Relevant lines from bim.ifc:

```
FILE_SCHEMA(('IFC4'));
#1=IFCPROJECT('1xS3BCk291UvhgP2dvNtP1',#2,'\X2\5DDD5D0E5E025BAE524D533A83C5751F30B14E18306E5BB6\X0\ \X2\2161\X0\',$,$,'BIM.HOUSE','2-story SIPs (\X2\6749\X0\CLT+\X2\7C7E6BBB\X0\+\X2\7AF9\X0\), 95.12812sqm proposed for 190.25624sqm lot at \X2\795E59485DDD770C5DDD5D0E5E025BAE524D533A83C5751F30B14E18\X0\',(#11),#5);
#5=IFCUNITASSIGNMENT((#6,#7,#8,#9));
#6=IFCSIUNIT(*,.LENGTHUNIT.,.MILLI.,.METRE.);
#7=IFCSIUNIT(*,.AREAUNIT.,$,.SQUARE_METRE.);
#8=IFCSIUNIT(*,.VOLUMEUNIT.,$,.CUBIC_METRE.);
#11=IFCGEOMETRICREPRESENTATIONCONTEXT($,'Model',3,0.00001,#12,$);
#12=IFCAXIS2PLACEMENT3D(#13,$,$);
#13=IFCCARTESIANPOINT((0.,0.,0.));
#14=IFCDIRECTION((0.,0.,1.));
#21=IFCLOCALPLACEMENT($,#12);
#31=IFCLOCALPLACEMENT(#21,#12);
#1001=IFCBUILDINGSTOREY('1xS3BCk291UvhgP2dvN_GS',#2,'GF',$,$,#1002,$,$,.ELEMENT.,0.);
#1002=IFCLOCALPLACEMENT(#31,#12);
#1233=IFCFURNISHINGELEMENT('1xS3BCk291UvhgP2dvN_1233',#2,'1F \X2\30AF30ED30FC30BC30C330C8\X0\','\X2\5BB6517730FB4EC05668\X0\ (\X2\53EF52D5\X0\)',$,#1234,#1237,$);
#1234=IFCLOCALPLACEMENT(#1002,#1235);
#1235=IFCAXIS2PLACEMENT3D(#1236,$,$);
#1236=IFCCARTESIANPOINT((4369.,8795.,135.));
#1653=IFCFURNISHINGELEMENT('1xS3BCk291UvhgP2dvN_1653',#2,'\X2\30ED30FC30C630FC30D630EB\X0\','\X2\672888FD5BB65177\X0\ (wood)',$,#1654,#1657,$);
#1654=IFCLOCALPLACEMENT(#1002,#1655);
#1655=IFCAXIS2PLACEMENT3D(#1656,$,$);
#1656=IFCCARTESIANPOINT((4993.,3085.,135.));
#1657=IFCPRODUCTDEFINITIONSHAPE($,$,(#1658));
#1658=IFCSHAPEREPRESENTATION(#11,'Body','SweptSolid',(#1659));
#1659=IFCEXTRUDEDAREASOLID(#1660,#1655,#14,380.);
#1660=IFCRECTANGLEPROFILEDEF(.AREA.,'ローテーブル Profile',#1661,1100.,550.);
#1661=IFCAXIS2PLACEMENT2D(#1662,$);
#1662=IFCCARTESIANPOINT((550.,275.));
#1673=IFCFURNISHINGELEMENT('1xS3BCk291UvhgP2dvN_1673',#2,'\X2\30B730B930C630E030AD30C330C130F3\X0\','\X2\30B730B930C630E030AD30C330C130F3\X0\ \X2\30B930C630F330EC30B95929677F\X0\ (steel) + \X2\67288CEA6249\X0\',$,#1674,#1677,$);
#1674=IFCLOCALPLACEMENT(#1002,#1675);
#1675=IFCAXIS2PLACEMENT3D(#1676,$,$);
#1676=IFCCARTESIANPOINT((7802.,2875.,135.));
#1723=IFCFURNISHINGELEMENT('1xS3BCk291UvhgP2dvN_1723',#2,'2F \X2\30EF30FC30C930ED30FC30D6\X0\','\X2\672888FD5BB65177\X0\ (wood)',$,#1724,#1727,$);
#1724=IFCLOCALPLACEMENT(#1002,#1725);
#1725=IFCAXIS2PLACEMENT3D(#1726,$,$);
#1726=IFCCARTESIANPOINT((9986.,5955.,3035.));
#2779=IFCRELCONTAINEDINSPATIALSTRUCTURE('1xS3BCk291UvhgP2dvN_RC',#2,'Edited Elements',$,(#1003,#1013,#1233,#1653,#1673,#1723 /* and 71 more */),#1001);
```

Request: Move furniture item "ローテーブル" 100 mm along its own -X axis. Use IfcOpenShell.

```python
import ifcopenshell
import ifcopenshell.api.geometry
import ifcopenshell.util.placement
import ifcopenshell.util.unit

model = ifcopenshell.open("bim.ifc")
unit_scale = ifcopenshell.util.unit.calculate_unit_scale(model)

item = model.by_id(1653)
matrix = ifcopenshell.util.placement.get_local_placement(item.ObjectPlacement)
matrix[:3, 3] -= matrix[:3, 0] * 0.1 / unit_scale
ifcopenshell.api.geometry.edit_object_placement(model, product=item, matrix=matrix, is_si=False)

print(ifcopenshell.util.placement.get_local_placement(item.ObjectPlacement).round(3) + 0.0)

model.write("bim-out.ifc")
```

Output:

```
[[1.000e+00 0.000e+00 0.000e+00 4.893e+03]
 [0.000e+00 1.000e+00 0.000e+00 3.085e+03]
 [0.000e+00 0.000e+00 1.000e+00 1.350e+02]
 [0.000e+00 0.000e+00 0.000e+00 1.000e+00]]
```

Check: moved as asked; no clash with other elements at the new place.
